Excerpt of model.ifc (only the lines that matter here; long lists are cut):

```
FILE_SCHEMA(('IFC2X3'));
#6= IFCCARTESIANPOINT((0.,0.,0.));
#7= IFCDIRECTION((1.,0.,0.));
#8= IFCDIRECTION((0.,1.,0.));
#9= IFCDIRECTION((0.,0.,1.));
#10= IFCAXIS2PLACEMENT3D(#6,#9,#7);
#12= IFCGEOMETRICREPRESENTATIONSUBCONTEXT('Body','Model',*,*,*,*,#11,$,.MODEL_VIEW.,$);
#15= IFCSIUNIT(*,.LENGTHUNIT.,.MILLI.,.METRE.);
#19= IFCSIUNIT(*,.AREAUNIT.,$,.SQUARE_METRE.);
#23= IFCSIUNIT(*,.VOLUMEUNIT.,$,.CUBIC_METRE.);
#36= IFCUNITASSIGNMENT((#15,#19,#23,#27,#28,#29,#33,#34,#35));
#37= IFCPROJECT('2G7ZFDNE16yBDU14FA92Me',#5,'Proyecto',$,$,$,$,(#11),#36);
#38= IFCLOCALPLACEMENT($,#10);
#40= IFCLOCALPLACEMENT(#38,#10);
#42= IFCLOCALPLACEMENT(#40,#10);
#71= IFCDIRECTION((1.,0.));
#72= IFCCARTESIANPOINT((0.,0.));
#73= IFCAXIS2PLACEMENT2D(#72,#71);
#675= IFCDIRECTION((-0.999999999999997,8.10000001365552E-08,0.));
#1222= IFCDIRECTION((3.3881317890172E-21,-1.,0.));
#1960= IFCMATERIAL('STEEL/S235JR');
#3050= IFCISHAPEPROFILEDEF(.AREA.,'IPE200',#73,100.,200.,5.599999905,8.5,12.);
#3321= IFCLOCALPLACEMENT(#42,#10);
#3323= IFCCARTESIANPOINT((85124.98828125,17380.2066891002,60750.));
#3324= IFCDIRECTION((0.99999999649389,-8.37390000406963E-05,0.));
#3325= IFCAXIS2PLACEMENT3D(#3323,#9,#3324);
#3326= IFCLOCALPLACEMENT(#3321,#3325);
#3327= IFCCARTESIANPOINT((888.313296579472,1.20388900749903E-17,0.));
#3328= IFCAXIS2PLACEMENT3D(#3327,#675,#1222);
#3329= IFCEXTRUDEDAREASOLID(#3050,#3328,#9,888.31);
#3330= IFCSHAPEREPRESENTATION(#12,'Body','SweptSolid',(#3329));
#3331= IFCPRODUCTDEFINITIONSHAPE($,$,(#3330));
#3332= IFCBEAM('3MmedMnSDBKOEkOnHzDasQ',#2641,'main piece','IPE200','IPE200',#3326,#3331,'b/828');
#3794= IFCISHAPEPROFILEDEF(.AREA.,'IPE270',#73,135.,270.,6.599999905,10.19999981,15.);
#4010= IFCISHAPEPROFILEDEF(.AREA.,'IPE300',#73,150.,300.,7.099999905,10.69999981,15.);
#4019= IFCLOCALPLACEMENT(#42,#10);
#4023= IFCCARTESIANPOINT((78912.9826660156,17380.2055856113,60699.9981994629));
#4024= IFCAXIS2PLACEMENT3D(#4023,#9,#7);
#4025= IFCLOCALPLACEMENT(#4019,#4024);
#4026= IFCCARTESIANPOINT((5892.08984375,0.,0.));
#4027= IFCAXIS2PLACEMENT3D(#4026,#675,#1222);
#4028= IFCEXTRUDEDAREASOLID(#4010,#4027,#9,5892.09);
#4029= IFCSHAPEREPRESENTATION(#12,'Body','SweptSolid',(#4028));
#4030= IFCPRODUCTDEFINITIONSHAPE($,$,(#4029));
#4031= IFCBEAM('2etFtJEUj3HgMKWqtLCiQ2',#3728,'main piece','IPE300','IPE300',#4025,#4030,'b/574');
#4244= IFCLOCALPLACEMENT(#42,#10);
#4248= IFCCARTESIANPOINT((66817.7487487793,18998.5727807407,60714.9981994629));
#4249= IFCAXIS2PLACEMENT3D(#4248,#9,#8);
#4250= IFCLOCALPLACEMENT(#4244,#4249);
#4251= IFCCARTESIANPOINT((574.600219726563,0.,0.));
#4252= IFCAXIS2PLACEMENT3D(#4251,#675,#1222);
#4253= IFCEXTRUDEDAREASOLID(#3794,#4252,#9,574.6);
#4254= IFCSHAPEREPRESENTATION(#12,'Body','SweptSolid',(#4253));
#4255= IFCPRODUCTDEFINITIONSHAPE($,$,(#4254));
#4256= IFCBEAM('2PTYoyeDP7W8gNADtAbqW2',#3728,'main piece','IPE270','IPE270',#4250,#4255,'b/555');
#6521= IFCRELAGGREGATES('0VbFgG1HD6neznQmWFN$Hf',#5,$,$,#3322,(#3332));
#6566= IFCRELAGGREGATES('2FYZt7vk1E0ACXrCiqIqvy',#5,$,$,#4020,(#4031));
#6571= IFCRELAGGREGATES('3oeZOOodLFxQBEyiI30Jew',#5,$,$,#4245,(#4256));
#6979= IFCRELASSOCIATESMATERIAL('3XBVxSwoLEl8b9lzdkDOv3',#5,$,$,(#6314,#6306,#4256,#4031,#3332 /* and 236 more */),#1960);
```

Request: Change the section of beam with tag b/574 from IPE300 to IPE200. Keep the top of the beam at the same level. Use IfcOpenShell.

```python
import ifcopenshell
import ifcopenshell.util.element
import ifcopenshell.util.representation

model = ifcopenshell.open("model.ifc")

member = model.by_guid("2etFtJEUj3HgMKWqtLCiQ2")
source = next(p for p in model.by_type("IfcIShapeProfileDef") if p.ProfileName == "IPE200")

body = ifcopenshell.util.representation.get_representation(member, "Model", "Body")
solid = body.Items[0]
old_profile = solid.SweptArea

# Copy the section's sizes but keep this member's own profile position.
profile = ifcopenshell.util.element.copy(model, source)
# Profiles are centred, so shift by half the change in depth to hold the top.
shift = (old_profile.OverallDepth - profile.OverallDepth) / 2
x, y = old_profile.Position.Location.Coordinates
up = (0.0, 1.0)  # upwards, in the solid's own plane
location = model.createIfcCartesianPoint((x + up[0] * shift, y + up[1] * shift))
profile.Position = model.createIfcAxis2Placement2D(location, old_profile.Position.RefDirection)
solid.SweptArea = profile
if not model.get_total_inverses(old_profile):
    ifcopenshell.util.element.remove_deep2(model, old_profile)
member.Description = member.Description.replace("IPE300", "IPE200")
member.ObjectType = member.ObjectType.replace("IPE300", "IPE200")

print(solid.SweptArea)

model.write("model_updated.ifc")
```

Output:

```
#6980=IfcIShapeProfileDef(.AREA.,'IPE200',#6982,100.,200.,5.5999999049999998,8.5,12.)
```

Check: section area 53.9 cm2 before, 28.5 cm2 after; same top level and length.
